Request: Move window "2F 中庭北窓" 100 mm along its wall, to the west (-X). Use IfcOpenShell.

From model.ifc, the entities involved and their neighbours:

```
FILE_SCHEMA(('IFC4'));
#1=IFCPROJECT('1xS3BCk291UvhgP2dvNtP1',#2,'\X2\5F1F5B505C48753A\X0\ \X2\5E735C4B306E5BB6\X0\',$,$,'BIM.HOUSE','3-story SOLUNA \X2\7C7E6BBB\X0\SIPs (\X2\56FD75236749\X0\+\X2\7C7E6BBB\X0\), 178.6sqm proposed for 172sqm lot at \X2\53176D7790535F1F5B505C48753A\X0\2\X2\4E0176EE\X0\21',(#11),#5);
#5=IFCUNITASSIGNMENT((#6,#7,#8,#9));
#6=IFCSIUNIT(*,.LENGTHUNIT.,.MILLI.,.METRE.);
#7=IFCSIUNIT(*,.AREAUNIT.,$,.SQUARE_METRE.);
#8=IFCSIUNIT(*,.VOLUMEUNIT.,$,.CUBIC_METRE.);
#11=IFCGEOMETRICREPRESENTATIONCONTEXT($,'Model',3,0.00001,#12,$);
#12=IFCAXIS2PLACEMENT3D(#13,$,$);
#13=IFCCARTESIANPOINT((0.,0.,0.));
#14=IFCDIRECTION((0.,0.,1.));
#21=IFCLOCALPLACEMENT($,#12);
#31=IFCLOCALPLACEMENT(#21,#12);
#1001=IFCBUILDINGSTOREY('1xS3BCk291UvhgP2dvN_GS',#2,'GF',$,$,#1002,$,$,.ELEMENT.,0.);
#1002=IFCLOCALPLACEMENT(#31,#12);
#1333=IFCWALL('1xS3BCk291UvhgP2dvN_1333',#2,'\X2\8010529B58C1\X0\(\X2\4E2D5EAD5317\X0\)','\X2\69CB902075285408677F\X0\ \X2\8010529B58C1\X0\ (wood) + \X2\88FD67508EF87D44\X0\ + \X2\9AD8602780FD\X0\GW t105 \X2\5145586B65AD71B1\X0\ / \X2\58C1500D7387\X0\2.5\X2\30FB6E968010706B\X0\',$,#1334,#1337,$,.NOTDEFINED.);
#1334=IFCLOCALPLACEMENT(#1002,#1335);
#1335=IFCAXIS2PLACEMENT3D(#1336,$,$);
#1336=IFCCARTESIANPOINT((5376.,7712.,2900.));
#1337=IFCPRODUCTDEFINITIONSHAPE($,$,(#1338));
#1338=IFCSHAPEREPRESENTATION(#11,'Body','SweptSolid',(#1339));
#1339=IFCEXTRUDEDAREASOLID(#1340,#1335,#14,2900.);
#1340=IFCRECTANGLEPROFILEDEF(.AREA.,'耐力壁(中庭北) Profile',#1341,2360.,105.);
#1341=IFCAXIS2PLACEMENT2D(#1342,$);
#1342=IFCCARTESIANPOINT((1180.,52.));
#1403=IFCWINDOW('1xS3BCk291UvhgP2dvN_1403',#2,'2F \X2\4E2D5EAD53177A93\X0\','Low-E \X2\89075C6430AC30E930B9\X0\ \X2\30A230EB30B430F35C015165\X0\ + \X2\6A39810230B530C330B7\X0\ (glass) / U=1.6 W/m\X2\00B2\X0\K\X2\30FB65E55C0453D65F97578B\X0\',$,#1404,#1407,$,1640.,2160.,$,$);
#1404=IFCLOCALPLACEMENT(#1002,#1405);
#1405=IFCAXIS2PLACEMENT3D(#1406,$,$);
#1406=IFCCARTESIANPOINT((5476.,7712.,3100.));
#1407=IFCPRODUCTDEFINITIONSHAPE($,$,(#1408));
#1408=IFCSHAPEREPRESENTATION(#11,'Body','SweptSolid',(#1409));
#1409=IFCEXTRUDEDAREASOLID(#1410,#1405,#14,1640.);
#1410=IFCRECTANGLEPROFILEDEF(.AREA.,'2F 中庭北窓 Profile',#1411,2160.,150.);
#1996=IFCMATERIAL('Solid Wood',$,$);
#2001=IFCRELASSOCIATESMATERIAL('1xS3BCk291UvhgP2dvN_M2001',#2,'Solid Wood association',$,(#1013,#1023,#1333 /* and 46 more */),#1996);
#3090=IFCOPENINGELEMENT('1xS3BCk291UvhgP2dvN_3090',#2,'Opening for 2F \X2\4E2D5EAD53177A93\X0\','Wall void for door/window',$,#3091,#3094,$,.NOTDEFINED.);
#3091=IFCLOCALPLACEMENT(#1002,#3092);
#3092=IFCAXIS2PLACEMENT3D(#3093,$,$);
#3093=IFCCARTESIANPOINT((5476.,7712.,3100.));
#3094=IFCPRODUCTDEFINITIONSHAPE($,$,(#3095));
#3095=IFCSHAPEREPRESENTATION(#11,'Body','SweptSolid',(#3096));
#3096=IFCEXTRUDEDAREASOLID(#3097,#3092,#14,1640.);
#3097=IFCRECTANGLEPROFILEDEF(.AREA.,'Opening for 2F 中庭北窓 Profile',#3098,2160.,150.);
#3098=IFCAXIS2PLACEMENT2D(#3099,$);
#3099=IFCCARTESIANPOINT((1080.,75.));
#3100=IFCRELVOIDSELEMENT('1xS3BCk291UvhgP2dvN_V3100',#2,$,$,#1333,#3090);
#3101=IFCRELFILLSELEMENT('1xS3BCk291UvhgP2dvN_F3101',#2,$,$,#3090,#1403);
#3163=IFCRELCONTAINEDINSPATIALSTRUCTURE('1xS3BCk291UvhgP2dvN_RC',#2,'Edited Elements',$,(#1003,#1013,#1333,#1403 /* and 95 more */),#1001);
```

```python
import ifcopenshell
import ifcopenshell.api.geometry
import ifcopenshell.util.placement
import ifcopenshell.util.unit

model = ifcopenshell.open("model.ifc")
unit_scale = ifcopenshell.util.unit.calculate_unit_scale(model)

window = model.by_guid("1xS3BCk291UvhgP2dvN_1403")
opening = window.FillsVoids[0].RelatingOpeningElement
wall = opening.VoidsElements[0].RelatingBuildingElement

wall_matrix = ifcopenshell.util.placement.get_local_placement(wall.ObjectPlacement)
shift = wall_matrix[:3, 0] * -0.1 / unit_scale
before = ifcopenshell.util.placement.get_local_placement(window.ObjectPlacement)[:3, 3].copy()

# The window is not placed relative to its opening, so move both.
for product in (opening, window):
    matrix = ifcopenshell.util.placement.get_local_placement(product.ObjectPlacement)
    matrix[:3, 3] += shift
    ifcopenshell.api.geometry.edit_object_placement(model, product=product, matrix=matrix, is_si=False)

after = ifcopenshell.util.placement.get_local_placement(window.ObjectPlacement)[:3, 3]
print("window moved by", (after - before).round(3) + 0.0)

model.write("model_rev.ifc")
```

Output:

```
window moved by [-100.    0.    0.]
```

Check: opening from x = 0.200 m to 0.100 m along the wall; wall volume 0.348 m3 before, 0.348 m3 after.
